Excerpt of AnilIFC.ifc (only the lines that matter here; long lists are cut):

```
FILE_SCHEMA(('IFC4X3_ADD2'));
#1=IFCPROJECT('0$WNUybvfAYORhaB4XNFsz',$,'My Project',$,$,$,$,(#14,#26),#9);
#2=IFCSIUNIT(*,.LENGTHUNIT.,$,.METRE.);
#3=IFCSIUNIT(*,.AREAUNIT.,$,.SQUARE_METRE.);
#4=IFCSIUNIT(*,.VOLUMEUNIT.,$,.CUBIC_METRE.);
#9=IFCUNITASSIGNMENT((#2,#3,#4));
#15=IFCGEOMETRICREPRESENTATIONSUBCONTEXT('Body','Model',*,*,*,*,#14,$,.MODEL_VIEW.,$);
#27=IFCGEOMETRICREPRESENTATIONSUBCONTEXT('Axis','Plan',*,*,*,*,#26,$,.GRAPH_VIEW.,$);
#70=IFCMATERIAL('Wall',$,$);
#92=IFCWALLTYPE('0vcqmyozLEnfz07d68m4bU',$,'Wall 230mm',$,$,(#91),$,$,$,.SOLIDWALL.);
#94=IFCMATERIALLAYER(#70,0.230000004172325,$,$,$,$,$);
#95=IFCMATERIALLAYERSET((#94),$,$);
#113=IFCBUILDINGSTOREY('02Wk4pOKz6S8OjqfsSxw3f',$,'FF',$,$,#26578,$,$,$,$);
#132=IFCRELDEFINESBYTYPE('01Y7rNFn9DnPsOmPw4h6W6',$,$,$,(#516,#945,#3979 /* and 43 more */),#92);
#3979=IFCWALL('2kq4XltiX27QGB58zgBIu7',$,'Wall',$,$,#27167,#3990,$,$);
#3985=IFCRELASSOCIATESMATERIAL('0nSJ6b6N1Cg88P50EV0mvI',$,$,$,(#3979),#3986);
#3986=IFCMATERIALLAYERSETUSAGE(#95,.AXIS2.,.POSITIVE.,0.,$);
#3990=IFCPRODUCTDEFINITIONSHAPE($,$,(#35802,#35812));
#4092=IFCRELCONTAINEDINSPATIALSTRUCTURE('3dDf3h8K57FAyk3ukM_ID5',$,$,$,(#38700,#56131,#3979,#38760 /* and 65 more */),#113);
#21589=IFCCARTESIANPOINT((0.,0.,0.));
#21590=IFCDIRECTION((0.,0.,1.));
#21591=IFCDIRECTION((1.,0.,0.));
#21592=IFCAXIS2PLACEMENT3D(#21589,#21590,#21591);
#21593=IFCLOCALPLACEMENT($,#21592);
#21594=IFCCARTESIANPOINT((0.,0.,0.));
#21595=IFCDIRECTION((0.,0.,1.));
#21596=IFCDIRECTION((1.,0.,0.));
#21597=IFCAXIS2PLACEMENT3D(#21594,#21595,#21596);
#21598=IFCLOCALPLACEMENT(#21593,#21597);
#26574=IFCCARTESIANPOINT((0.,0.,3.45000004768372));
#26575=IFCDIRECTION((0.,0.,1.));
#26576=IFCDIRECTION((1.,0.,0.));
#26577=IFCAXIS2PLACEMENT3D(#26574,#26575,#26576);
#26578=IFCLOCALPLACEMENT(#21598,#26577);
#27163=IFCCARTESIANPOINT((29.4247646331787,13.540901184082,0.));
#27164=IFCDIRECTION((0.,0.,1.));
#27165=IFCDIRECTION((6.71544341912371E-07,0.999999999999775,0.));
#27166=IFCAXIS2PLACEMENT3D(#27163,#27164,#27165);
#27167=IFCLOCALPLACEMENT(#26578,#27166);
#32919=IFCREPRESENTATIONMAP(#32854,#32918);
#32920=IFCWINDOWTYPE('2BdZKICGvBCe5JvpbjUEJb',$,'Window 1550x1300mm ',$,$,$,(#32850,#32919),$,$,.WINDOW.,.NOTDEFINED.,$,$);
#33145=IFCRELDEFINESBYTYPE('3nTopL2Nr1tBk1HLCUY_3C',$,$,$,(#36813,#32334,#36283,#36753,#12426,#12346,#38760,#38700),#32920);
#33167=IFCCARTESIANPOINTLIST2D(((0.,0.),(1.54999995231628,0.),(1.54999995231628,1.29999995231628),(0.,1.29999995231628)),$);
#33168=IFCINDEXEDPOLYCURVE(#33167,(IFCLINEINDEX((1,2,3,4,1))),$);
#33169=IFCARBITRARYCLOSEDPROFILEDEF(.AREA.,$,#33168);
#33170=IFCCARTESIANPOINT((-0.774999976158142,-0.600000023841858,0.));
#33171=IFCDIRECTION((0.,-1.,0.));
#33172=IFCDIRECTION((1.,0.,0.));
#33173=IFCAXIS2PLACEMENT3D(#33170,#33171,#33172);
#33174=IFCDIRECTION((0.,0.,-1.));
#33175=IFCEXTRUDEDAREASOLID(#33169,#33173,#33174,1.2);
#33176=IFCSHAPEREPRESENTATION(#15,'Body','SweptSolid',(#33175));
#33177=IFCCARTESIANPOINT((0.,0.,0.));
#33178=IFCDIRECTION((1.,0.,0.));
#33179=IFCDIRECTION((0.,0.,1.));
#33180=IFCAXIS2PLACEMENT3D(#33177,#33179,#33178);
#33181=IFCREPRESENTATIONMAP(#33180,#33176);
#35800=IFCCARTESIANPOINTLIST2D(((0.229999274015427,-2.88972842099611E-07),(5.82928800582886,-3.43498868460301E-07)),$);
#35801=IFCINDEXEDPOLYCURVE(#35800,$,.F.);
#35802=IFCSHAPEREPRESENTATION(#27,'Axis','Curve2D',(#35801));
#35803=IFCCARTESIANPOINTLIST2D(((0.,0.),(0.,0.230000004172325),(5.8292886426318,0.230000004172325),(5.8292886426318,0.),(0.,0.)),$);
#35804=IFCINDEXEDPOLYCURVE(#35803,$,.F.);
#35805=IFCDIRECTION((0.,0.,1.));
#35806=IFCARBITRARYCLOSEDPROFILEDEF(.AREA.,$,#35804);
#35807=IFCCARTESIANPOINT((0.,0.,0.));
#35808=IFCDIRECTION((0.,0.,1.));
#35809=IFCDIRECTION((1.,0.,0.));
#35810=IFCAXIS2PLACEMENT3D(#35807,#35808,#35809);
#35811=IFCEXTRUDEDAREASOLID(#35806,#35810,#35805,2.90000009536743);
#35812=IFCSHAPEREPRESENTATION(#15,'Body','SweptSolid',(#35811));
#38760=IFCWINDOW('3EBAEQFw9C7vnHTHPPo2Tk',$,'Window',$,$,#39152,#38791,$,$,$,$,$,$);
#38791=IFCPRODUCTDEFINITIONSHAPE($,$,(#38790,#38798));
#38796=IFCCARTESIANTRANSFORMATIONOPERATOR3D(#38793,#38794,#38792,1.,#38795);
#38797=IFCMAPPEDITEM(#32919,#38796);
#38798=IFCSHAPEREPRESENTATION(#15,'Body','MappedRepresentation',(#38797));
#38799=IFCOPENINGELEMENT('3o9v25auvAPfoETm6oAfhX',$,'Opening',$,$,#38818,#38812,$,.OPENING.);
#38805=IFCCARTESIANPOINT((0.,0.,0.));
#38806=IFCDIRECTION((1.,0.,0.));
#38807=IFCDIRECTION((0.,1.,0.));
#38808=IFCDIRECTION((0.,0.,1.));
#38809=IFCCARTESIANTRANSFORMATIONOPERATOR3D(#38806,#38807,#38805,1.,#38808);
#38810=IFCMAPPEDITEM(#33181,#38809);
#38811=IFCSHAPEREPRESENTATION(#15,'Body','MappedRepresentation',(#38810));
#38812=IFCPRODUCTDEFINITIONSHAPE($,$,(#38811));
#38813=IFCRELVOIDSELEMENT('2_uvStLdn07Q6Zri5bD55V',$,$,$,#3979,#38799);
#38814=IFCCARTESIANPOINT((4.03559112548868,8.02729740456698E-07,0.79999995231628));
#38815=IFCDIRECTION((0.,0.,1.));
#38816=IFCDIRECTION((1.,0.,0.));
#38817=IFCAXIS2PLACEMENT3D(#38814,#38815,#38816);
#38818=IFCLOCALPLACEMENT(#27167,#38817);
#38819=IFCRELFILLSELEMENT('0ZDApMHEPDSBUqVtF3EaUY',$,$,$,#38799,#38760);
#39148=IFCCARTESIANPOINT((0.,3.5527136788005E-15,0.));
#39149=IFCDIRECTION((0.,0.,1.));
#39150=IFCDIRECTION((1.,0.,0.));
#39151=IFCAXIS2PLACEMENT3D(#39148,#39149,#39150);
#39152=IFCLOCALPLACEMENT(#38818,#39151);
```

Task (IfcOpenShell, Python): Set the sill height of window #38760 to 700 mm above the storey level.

```python
import numpy as np
import ifcopenshell
import ifcopenshell.api.geometry
import ifcopenshell.geom
import ifcopenshell.util.element
import ifcopenshell.util.placement
import ifcopenshell.util.shape
import ifcopenshell.util.unit

model = ifcopenshell.open("AnilIFC.ifc")
unit_scale = ifcopenshell.util.unit.calculate_unit_scale(model)

window = model.by_guid("3EBAEQFw9C7vnHTHPPo2Tk")
opening = window.FillsVoids[0].RelatingOpeningElement
storey = ifcopenshell.util.element.get_container(window, ifc_class="IfcBuildingStorey")
level = ifcopenshell.util.placement.get_local_placement(storey.ObjectPlacement)[2, 3]

# The opening's origin need not be at the sill, so measure its lowest point.
shape = ifcopenshell.geom.create_shape(ifcopenshell.geom.settings(), opening)
bottom = ifcopenshell.util.shape.get_shape_bottom_elevation(shape, shape.geometry) / unit_scale
dz = level + 0.7 / unit_scale - bottom

shift = np.array([0.0, 0.0, dz])
# The window is placed relative to its opening, so it follows when the opening moves.
matrix = ifcopenshell.util.placement.get_local_placement(opening.ObjectPlacement)
matrix[:3, 3] += shift
ifcopenshell.api.geometry.edit_object_placement(
    model, product=opening, matrix=matrix, is_si=False, should_transform_children=True
)

print(f"moved by {dz * unit_scale:+.3f} m")

model.write("AnilIFC-out.ifc")
```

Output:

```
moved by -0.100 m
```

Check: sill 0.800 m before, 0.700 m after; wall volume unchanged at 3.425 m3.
